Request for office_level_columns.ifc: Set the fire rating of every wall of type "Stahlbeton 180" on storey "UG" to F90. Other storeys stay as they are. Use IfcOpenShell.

First a look at what the model holds.

```python
import ifcopenshell
import ifcopenshell.util.element

model = ifcopenshell.open("office_level_columns.ifc")
print(model.schema)
storey = next(s for s in model.by_type("IfcBuildingStorey") if s.Name == "UG")
walls = [e for e in ifcopenshell.util.element.get_decomposition(storey) if e.is_a("IfcWall")]
seen = {}
for e in walls:
    element_type = ifcopenshell.util.element.get_type(e)
    key = (element_type.Name if element_type != e and element_type else None, ifcopenshell.util.element.get_pset(e, "Pset_WallCommon", "FireRating"))
    seen[key] = seen.get(key, 0) + 1
for (name, value), count in sorted(seen.items(), key=str):
    print(count, "x", name, "|", value)
```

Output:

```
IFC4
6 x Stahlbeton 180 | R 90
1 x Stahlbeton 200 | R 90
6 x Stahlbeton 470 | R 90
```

```python
import ifcopenshell
import ifcopenshell.api.pset
import ifcopenshell.util.element

model = ifcopenshell.open("office_level_columns.ifc")

storey = next(s for s in model.by_type("IfcBuildingStorey") if s.Name == "UG")
walls = [e for e in ifcopenshell.util.element.get_decomposition(storey) if e.is_a("IfcWall")]

count = 0
for e in walls:
    element_type = ifcopenshell.util.element.get_type(e)
    if element_type in (None, e) or element_type.Name != "Stahlbeton 180":
        continue
    # add_pset returns the element's existing set when there is one.
    pset = ifcopenshell.api.pset.add_pset(model, product=e, name="Pset_WallCommon")
    ifcopenshell.api.pset.edit_pset(model, pset=pset, properties={"FireRating": "F90"})
    count += 1

print(count, "walls updated")

model.write("office_level_columns_edited.ifc")
```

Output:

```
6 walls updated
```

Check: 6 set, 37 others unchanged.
